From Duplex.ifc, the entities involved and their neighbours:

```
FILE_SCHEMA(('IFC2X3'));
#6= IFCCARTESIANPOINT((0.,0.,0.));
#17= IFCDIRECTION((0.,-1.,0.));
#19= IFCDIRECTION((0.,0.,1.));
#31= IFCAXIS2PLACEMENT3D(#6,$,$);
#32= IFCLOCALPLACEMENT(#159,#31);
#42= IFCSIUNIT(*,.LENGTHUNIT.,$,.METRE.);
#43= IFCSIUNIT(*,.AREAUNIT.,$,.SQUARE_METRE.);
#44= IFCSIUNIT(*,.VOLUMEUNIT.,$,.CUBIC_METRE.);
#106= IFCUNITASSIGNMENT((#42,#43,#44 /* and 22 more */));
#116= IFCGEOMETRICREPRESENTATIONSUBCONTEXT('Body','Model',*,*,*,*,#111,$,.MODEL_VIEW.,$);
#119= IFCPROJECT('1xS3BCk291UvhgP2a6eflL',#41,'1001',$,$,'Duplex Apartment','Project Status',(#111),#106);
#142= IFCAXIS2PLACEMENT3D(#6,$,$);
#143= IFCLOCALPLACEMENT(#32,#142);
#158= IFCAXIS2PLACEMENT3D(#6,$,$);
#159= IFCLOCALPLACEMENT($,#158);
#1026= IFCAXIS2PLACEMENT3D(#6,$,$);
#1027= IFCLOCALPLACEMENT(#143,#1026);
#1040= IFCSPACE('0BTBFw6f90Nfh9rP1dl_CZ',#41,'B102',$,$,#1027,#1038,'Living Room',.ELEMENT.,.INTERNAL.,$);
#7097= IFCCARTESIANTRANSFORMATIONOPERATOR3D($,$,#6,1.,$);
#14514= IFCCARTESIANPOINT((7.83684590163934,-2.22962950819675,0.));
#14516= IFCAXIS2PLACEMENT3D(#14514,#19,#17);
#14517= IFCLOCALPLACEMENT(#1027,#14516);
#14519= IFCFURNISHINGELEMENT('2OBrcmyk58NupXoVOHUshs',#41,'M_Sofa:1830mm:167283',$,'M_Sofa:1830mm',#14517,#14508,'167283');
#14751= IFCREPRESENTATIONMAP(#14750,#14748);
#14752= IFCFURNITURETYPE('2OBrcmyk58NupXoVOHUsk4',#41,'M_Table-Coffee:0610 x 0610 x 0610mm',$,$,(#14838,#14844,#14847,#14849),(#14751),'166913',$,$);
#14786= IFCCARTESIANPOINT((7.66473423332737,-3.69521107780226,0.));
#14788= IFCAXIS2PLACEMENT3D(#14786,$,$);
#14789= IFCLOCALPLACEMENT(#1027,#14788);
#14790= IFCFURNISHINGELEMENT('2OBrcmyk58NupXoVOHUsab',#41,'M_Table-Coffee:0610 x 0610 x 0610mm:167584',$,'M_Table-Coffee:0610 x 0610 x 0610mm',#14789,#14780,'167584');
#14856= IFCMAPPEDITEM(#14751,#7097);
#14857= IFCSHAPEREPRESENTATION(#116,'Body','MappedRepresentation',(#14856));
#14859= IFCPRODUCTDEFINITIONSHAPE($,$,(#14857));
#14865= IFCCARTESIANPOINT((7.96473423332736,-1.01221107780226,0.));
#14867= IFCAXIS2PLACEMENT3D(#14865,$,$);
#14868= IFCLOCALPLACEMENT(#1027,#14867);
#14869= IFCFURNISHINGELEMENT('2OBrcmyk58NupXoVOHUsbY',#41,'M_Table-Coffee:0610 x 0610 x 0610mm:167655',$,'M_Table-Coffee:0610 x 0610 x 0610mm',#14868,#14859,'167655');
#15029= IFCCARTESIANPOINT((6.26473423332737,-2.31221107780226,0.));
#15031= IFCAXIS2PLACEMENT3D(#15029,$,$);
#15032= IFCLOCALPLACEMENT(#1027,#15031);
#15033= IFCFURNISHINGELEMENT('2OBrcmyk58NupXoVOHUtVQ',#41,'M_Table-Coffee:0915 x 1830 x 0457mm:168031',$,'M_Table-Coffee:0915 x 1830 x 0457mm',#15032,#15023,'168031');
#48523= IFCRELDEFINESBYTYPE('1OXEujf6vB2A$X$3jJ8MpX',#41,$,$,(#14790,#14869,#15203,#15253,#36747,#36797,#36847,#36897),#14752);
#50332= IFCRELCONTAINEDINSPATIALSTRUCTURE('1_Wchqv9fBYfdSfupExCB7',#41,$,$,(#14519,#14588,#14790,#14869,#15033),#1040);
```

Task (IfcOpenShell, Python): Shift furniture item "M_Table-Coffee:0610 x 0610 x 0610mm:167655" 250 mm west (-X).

```python
import ifcopenshell
import ifcopenshell.api.geometry
import ifcopenshell.util.placement

model = ifcopenshell.open("Duplex.ifc")

item = model.by_id(14869)
matrix = ifcopenshell.util.placement.get_local_placement(item.ObjectPlacement)
matrix[0, 3] -= 0.25
ifcopenshell.api.geometry.edit_object_placement(model, product=item, matrix=matrix, is_si=False)

print(ifcopenshell.util.placement.get_local_placement(item.ObjectPlacement).round(3) + 0.0)

model.write("Duplex_edited.ifc")
```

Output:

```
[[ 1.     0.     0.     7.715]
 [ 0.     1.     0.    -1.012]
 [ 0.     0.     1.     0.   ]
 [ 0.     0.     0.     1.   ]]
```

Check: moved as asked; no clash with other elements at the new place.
